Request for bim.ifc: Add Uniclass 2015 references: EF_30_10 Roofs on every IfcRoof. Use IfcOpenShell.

First a look at what the model holds.

```python
import ifcopenshell

model = ifcopenshell.open("bim.ifc")
print(model.schema)
print("classifications:", [c.Name for c in model.by_type("IfcClassification")])
for ifc_class in ("IfcDoor", "IfcRoof", "IfcStair", "IfcWall", "IfcWindow"):
    print(ifc_class, len(model.by_type(ifc_class)))
```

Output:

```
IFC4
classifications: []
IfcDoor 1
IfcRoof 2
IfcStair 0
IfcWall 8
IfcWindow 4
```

```python
import ifcopenshell
import ifcopenshell.api.classification

model = ifcopenshell.open("bim.ifc")

system = ifcopenshell.api.classification.add_classification(model, classification="Uniclass 2015")

codes = {
    "IfcRoof": ("EF_30_10", "Roofs"),
}
for ifc_class, (code, name) in codes.items():
    products = model.by_type(ifc_class)
    ifcopenshell.api.classification.add_reference(
        model, products=products, classification=system, identification=code, name=name
    )
    print(code, len(products))

model.write("bim_updated.ifc")
```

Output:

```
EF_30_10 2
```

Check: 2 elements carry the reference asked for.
